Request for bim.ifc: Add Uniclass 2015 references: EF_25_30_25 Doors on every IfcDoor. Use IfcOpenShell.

First a look at what the model holds.

```python
import ifcopenshell

model = ifcopenshell.open("bim.ifc")
print(model.schema)
print("classifications:", [c.Name for c in model.by_type("IfcClassification")])
for ifc_class in ("IfcDoor", "IfcRoof", "IfcStair", "IfcWall", "IfcWindow"):
    print(ifc_class, len(model.by_type(ifc_class)))
```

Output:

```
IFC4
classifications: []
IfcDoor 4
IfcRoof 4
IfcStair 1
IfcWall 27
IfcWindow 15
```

```python
import ifcopenshell
import ifcopenshell.api.classification

model = ifcopenshell.open("bim.ifc")

system = ifcopenshell.api.classification.add_classification(model, classification="Uniclass 2015")

codes = {
    "IfcDoor": ("EF_25_30_25", "Doors"),
}
for ifc_class, (code, name) in codes.items():
    products = model.by_type(ifc_class)
    ifcopenshell.api.classification.add_reference(
        model, products=products, classification=system, identification=code, name=name
    )
    print(code, len(products))

model.write("bim_edited.ifc")
```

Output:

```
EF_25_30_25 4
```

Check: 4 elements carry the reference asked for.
